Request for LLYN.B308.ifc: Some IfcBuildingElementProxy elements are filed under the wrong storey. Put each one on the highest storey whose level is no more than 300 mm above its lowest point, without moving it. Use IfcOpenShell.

First a look at what the model holds.

```python
import ifcopenshell
import ifcopenshell.util.element
import ifcopenshell.util.placement

model = ifcopenshell.open("LLYN.B308.ifc")
print(model.schema)
for storey in model.by_type("IfcBuildingStorey"):
    level = ifcopenshell.util.placement.get_storey_elevation(storey)
    count = sum(e.is_a("IfcBuildingElementProxy") for e in ifcopenshell.util.element.get_contained(storey))
    print(storey.id(), storey.Name, round(level, 3), count, sep=" | ")
```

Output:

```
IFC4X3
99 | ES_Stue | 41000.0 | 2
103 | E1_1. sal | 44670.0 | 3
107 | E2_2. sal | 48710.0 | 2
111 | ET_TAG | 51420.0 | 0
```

```python
import ifcopenshell
import ifcopenshell.api.spatial
import ifcopenshell.geom
import ifcopenshell.util.element
import ifcopenshell.util.placement
import ifcopenshell.util.shape
import ifcopenshell.util.unit

model = ifcopenshell.open("LLYN.B308.ifc")
unit_scale = ifcopenshell.util.unit.calculate_unit_scale(model)
settings = ifcopenshell.geom.settings()

levels = sorted(
    ((ifcopenshell.util.placement.get_storey_elevation(s) * unit_scale, s) for s in model.by_type("IfcBuildingStorey")),
    key=lambda pair: pair[0],
)

for e in model.by_type("IfcBuildingElementProxy"):
    current = e.ContainedInStructure[0].RelatingStructure if e.ContainedInStructure else None
    if current is None or not current.is_a("IfcBuildingStorey"):
        continue
    shape = ifcopenshell.geom.create_shape(settings, e)
    bottom = ifcopenshell.util.shape.get_shape_bottom_elevation(shape, shape.geometry)
    below = [s for level, s in levels if level <= bottom + 0.3]
    storey = below[-1] if below else levels[0][1]
    if storey != current:
        # assign_container keeps the world position.
        ifcopenshell.api.spatial.assign_container(model, products=[e], relating_structure=storey)
        print(e.id(), current.Name, "->", storey.Name)

model.write("LLYN.B308_rev.ifc")
```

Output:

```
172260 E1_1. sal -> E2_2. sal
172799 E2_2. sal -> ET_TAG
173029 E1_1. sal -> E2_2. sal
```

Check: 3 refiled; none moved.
